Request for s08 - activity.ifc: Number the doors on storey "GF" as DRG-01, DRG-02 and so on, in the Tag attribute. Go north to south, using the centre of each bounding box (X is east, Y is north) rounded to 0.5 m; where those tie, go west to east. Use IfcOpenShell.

First a look at what the model holds.

```python
import ifcopenshell
import ifcopenshell.util.element
import ifcopenshell.util.placement

model = ifcopenshell.open("s08 - activity.ifc")
print(model.schema)
storey = next(s for s in model.by_type("IfcBuildingStorey") if s.Name == "GF")
doors = [e for e in ifcopenshell.util.element.get_decomposition(storey) if e.is_a("IfcDoor")]
for e in sorted(doors, key=lambda e: e.id()):
    origin = ifcopenshell.util.placement.get_local_placement(e.ObjectPlacement)[:3, 3]
    print(e.id(), e.Tag, e.Name, origin.round(2) + 0.0, sep=" | ")
```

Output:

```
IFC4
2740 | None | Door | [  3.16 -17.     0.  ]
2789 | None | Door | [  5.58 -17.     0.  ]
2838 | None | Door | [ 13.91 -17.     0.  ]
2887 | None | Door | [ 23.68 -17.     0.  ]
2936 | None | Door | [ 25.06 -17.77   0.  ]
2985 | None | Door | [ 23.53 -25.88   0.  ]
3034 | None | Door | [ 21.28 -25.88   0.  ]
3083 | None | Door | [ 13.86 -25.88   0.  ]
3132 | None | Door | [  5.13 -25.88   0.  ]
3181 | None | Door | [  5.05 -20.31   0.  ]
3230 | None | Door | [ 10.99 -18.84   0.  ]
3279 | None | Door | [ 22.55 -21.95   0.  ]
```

```python
import ifcopenshell
import ifcopenshell.geom
import ifcopenshell.util.element
import ifcopenshell.util.shape

model = ifcopenshell.open("s08 - activity.ifc")
settings = ifcopenshell.geom.settings()
settings.set("use-world-coords", True)


def centre(element):
    shape = ifcopenshell.geom.create_shape(settings, element)
    return ifcopenshell.util.shape.get_bbox_centroid(shape.geometry)


storey = next(s for s in model.by_type("IfcBuildingStorey") if s.Name == "GF")
doors = [e for e in ifcopenshell.util.element.get_decomposition(storey) if e.is_a("IfcDoor")]

# Insertion points can sit at a corner or the storey origin, so sort by the geometry (in metres).
centres = {e: centre(e) for e in doors}
doors.sort(key=lambda e: (-round(centres[e][1] / 0.5), centres[e][0]))

for i, e in enumerate(doors, start=1):
    number = f"DRG-{i:02d}"
    e.Tag = number
    print(e.id(), number)

model.write("s08 - activity_v2.ifc")
```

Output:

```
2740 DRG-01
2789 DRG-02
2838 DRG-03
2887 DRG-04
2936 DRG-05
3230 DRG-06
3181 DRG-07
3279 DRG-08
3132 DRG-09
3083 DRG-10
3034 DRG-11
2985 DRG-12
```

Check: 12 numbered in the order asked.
